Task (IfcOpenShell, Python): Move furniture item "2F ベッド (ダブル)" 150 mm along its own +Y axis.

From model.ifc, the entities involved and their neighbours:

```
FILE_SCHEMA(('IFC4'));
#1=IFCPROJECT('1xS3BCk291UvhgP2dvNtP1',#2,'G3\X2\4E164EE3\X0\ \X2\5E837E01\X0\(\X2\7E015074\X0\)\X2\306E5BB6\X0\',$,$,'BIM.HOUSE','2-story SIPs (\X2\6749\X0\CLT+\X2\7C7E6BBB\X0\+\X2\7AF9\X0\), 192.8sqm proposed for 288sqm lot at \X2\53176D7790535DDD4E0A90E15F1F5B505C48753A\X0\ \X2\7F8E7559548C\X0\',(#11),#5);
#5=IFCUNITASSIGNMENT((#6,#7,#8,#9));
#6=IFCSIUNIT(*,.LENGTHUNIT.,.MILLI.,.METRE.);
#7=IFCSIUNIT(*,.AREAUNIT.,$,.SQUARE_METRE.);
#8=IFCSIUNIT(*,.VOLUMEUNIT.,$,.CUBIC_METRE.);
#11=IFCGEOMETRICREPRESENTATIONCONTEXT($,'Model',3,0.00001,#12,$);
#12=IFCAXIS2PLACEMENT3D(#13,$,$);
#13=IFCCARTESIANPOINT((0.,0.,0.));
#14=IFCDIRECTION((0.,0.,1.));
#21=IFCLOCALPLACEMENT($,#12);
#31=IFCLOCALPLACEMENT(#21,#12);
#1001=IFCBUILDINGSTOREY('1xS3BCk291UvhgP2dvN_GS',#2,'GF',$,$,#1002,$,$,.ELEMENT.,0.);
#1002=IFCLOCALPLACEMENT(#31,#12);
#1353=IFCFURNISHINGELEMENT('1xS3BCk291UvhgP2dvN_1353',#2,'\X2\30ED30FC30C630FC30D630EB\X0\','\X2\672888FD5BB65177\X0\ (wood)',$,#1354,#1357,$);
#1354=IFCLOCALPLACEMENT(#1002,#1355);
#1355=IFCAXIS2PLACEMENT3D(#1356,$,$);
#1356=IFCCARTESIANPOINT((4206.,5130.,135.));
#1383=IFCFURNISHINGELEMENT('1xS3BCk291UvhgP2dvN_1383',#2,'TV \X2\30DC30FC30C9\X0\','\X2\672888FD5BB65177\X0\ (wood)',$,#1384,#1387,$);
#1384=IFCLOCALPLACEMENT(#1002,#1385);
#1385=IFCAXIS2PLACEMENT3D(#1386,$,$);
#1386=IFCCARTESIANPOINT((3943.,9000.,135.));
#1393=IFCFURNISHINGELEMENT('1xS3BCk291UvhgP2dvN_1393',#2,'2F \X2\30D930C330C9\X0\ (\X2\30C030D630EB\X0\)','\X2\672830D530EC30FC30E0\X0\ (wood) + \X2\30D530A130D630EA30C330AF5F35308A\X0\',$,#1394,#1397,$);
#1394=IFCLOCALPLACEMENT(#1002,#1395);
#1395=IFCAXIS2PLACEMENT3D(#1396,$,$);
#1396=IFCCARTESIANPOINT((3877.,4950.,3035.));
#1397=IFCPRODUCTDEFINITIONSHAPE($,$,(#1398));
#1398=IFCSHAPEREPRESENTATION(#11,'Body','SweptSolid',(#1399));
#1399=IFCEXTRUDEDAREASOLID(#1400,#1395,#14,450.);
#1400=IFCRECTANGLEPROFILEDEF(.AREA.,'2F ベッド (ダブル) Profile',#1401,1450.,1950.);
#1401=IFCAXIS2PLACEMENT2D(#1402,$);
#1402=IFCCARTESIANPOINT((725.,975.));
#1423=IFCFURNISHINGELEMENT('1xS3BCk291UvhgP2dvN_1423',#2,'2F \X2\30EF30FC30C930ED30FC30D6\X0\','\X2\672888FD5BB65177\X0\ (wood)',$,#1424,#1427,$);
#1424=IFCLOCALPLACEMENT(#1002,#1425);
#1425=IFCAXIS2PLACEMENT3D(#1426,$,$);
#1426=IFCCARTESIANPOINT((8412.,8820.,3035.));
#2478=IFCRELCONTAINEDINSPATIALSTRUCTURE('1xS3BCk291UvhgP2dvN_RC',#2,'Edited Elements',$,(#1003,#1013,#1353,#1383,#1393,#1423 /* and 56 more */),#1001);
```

```python
import ifcopenshell
import ifcopenshell.api.geometry
import ifcopenshell.util.placement
import ifcopenshell.util.unit

model = ifcopenshell.open("model.ifc")
unit_scale = ifcopenshell.util.unit.calculate_unit_scale(model)

item = model.by_guid("1xS3BCk291UvhgP2dvN_1393")
matrix = ifcopenshell.util.placement.get_local_placement(item.ObjectPlacement)
matrix[:3, 3] += matrix[:3, 1] * 0.15 / unit_scale
ifcopenshell.api.geometry.edit_object_placement(model, product=item, matrix=matrix, is_si=False)

print(ifcopenshell.util.placement.get_local_placement(item.ObjectPlacement).round(3) + 0.0)

model.write("model-out.ifc")
```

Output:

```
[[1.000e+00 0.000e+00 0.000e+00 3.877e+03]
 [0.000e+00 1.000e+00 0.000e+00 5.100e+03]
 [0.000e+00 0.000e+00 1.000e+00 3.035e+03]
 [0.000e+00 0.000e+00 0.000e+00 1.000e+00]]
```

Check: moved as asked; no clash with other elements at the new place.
